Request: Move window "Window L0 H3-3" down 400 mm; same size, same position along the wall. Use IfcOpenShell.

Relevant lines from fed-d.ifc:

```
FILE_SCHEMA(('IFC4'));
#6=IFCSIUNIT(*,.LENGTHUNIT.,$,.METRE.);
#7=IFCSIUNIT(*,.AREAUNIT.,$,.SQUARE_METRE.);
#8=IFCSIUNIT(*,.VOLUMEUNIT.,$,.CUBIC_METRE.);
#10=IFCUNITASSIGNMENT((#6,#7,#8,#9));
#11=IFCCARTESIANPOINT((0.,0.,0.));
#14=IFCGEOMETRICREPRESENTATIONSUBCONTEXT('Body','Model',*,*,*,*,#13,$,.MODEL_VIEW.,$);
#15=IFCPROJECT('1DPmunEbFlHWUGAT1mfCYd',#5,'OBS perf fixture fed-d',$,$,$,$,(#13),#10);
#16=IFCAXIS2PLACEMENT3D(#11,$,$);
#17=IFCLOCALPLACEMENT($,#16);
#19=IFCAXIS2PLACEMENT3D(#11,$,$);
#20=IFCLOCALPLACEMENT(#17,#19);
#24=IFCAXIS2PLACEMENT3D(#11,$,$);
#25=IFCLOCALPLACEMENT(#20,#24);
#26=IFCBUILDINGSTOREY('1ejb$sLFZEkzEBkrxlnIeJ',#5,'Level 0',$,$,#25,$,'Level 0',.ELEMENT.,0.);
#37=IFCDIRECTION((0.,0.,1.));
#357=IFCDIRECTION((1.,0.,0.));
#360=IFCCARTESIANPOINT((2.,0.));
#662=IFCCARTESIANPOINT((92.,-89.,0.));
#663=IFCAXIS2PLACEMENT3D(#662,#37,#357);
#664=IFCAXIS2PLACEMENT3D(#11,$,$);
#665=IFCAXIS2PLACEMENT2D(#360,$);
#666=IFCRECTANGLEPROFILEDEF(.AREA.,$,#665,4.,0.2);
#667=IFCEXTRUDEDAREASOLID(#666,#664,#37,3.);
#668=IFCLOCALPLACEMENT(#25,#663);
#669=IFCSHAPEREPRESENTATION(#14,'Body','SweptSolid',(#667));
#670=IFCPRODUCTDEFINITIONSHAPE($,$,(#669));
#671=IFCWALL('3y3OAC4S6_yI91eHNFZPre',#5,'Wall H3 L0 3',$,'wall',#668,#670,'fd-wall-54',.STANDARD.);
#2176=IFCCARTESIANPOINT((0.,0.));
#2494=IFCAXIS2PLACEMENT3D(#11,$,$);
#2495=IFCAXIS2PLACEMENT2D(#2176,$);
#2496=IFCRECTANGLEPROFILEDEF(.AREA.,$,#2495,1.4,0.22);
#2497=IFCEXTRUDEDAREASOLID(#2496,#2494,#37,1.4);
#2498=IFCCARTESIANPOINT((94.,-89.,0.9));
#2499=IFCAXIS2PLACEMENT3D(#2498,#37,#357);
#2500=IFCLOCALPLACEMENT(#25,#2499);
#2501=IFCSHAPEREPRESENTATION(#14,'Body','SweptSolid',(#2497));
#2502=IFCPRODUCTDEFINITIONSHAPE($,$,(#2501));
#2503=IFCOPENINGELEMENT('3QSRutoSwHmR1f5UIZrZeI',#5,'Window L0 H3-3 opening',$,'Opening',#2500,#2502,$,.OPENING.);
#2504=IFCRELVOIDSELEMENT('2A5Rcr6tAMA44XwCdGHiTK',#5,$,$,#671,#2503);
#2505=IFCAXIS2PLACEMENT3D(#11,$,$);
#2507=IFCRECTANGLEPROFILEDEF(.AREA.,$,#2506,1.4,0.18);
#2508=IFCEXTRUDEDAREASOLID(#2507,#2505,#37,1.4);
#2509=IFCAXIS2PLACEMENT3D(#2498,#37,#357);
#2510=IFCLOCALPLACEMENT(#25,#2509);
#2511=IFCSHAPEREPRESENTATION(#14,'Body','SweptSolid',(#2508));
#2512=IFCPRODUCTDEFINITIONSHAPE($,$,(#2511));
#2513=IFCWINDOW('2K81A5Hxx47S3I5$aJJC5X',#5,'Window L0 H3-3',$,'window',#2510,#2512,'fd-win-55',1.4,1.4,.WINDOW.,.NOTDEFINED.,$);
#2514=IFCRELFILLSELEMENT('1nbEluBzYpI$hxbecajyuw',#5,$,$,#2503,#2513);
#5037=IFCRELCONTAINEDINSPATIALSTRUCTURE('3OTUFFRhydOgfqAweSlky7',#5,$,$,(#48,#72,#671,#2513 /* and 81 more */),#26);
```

```python
import numpy as np
import ifcopenshell
import ifcopenshell.api.geometry
import ifcopenshell.util.placement
import ifcopenshell.util.unit

model = ifcopenshell.open("fed-d.ifc")
unit_scale = ifcopenshell.util.unit.calculate_unit_scale(model)

window = model.by_id(2513)
opening = window.FillsVoids[0].RelatingOpeningElement
dz = -0.4 / unit_scale

shift = np.array([0.0, 0.0, dz])
# The window is not placed relative to its opening, so move both.
for product in (opening, window):
    matrix = ifcopenshell.util.placement.get_local_placement(product.ObjectPlacement)
    matrix[:3, 3] += shift
    ifcopenshell.api.geometry.edit_object_placement(model, product=product, matrix=matrix, is_si=False)

print(f"moved by {dz * unit_scale:+.3f} m")

model.write("fed-d_v2.ifc")
```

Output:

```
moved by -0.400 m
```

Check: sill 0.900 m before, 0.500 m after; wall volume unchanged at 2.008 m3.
